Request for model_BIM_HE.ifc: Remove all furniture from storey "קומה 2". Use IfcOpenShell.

First a look at what the model holds.

```python
import ifcopenshell
import ifcopenshell.util.element

model = ifcopenshell.open("model_BIM_HE.ifc")
print(model.schema)
storey = next(s for s in model.by_type("IfcBuildingStorey") if s.Name == "קומה 2")
furniture = [e for e in ifcopenshell.util.element.get_decomposition(storey) if e.is_a("IfcFurnishingElement")]
seen = {}
for e in furniture:
    element_type = ifcopenshell.util.element.get_type(e)
    name = element_type.Name if element_type not in (None, e) else None
    seen[name] = seen.get(name, 0) + 1
for name, count in sorted(seen.items(), key=str):
    print(count, "x", name)
```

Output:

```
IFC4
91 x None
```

```python
import ifcopenshell
import ifcopenshell.api.root
import ifcopenshell.util.element

model = ifcopenshell.open("model_BIM_HE.ifc")

storey = next(s for s in model.by_type("IfcBuildingStorey") if s.Name == "קומה 2")
furniture = [e for e in ifcopenshell.util.element.get_decomposition(storey) if e.is_a("IfcFurnishingElement")]

for e in furniture:
    ifcopenshell.api.root.remove_product(model, product=e)
print(len(furniture), "removed")

model.write("model_BIM_HE_rev.ifc")
```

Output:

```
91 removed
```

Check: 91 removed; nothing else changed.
